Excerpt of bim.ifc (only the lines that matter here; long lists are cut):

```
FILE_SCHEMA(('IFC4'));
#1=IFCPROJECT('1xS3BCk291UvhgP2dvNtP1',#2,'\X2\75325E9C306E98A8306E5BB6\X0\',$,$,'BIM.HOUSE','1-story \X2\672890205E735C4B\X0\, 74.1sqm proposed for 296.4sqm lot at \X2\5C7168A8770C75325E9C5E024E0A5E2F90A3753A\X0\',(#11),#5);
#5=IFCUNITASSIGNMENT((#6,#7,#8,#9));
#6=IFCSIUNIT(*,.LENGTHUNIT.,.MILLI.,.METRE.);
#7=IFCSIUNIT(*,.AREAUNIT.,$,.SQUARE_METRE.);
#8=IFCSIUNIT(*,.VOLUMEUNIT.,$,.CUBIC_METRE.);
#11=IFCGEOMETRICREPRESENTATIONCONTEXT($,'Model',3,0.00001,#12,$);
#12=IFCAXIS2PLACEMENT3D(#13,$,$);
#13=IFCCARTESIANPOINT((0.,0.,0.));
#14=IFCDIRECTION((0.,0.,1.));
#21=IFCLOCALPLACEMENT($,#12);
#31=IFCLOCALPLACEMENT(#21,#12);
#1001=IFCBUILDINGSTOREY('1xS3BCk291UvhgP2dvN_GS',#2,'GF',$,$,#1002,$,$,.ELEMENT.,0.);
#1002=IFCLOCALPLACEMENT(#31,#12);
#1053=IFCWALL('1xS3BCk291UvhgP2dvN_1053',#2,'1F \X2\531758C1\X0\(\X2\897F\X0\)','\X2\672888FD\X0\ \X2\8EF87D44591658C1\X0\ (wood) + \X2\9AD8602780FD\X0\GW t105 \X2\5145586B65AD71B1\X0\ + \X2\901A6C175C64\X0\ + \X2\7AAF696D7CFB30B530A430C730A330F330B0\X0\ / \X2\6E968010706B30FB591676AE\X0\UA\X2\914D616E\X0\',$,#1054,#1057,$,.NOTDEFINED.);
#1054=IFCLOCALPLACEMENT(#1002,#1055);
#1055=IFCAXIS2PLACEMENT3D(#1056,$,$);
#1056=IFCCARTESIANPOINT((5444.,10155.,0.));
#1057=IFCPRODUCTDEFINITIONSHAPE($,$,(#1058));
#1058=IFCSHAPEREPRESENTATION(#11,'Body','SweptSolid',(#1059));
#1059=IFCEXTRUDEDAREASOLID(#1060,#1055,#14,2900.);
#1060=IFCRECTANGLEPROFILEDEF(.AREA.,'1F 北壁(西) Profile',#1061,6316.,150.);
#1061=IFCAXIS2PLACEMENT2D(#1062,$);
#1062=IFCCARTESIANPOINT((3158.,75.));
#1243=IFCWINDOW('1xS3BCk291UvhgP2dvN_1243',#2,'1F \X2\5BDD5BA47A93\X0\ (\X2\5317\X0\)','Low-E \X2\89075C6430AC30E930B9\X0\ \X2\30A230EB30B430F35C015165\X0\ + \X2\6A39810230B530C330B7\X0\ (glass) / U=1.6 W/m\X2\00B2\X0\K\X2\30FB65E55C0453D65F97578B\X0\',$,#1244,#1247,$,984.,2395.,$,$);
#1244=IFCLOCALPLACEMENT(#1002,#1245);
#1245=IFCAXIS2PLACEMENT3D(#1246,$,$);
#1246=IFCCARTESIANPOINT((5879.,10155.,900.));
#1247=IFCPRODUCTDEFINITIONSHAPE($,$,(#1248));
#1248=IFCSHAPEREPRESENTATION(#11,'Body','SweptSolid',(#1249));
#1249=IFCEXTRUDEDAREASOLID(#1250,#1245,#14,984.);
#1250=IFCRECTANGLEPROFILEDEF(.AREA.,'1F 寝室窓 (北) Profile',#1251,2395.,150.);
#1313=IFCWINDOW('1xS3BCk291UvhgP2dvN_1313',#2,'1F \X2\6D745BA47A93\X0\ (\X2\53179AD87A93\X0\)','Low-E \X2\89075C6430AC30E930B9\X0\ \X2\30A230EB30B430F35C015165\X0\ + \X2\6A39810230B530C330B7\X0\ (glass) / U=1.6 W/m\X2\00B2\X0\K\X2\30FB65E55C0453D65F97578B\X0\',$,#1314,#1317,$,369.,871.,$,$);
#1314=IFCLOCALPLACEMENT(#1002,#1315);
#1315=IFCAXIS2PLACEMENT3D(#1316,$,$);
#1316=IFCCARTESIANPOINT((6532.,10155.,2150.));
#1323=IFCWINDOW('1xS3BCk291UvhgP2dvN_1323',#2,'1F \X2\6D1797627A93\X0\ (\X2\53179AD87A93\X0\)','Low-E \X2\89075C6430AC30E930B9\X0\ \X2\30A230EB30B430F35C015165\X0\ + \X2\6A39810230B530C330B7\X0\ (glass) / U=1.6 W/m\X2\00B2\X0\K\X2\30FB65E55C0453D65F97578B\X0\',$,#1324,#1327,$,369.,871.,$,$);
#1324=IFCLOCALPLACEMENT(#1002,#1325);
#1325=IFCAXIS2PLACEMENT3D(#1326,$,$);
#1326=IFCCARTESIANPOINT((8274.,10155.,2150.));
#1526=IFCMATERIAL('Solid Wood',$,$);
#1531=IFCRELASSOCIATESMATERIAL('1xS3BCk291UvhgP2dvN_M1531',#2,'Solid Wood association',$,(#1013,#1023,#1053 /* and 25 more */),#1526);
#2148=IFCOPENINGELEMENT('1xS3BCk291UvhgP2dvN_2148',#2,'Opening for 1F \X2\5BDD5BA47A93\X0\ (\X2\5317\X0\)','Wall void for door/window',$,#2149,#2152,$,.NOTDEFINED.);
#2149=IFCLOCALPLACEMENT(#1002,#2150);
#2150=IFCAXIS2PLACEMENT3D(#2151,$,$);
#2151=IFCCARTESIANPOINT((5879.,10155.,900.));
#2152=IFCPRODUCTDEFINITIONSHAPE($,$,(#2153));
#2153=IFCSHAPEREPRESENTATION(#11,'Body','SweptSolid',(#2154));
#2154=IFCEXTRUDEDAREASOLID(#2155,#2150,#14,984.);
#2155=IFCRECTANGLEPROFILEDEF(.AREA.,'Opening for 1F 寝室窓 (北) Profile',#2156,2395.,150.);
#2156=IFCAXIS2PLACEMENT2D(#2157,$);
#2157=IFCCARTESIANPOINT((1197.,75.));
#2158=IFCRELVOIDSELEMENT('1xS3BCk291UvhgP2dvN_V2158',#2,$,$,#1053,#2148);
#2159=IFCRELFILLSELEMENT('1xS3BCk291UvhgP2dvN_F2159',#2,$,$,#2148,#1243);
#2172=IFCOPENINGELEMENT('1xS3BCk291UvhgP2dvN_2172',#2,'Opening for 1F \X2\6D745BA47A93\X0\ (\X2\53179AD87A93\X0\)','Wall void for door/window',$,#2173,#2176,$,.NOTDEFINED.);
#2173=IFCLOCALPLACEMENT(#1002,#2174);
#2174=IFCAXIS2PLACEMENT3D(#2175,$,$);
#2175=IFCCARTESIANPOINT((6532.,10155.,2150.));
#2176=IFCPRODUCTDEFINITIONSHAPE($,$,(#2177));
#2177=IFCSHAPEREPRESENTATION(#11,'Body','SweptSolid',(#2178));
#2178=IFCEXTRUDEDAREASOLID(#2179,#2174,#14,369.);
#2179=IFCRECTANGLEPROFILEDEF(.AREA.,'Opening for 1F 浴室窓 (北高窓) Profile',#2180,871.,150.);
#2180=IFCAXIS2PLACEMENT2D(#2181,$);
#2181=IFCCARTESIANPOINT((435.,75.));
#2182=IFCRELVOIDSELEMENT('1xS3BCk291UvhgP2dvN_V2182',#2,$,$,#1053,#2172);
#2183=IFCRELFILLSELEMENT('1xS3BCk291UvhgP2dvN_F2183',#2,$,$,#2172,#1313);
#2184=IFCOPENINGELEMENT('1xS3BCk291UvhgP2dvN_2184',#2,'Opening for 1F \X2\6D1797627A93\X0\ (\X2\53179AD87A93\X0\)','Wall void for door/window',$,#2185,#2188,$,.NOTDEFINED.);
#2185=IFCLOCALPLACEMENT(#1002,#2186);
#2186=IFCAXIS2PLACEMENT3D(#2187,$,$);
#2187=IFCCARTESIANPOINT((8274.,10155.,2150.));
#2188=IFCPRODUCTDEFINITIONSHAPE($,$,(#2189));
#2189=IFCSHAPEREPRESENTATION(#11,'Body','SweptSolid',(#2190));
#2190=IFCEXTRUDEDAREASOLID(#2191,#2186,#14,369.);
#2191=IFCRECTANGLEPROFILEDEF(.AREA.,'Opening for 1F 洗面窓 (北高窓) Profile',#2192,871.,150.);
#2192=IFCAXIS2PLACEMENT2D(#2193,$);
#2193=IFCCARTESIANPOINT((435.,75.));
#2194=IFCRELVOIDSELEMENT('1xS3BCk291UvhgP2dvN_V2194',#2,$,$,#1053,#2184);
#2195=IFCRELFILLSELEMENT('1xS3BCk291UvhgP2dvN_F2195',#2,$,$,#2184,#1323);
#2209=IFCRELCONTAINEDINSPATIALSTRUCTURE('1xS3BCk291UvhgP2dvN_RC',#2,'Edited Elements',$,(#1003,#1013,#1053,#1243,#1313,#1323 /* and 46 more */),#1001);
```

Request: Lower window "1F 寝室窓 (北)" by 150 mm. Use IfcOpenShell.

```python
import numpy as np
import ifcopenshell
import ifcopenshell.api.geometry
import ifcopenshell.util.placement
import ifcopenshell.util.unit

model = ifcopenshell.open("bim.ifc")
unit_scale = ifcopenshell.util.unit.calculate_unit_scale(model)

window = model.by_guid("1xS3BCk291UvhgP2dvN_1243")
opening = window.FillsVoids[0].RelatingOpeningElement
dz = -0.15 / unit_scale

shift = np.array([0.0, 0.0, dz])
# The window is not placed relative to its opening, so move both.
for product in (opening, window):
    matrix = ifcopenshell.util.placement.get_local_placement(product.ObjectPlacement)
    matrix[:3, 3] += shift
    ifcopenshell.api.geometry.edit_object_placement(model, product=product, matrix=matrix, is_si=False)

print(f"moved by {dz * unit_scale:+.3f} m")

model.write("bim_updated.ifc")
```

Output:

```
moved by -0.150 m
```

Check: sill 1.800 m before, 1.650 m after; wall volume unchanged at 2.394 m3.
